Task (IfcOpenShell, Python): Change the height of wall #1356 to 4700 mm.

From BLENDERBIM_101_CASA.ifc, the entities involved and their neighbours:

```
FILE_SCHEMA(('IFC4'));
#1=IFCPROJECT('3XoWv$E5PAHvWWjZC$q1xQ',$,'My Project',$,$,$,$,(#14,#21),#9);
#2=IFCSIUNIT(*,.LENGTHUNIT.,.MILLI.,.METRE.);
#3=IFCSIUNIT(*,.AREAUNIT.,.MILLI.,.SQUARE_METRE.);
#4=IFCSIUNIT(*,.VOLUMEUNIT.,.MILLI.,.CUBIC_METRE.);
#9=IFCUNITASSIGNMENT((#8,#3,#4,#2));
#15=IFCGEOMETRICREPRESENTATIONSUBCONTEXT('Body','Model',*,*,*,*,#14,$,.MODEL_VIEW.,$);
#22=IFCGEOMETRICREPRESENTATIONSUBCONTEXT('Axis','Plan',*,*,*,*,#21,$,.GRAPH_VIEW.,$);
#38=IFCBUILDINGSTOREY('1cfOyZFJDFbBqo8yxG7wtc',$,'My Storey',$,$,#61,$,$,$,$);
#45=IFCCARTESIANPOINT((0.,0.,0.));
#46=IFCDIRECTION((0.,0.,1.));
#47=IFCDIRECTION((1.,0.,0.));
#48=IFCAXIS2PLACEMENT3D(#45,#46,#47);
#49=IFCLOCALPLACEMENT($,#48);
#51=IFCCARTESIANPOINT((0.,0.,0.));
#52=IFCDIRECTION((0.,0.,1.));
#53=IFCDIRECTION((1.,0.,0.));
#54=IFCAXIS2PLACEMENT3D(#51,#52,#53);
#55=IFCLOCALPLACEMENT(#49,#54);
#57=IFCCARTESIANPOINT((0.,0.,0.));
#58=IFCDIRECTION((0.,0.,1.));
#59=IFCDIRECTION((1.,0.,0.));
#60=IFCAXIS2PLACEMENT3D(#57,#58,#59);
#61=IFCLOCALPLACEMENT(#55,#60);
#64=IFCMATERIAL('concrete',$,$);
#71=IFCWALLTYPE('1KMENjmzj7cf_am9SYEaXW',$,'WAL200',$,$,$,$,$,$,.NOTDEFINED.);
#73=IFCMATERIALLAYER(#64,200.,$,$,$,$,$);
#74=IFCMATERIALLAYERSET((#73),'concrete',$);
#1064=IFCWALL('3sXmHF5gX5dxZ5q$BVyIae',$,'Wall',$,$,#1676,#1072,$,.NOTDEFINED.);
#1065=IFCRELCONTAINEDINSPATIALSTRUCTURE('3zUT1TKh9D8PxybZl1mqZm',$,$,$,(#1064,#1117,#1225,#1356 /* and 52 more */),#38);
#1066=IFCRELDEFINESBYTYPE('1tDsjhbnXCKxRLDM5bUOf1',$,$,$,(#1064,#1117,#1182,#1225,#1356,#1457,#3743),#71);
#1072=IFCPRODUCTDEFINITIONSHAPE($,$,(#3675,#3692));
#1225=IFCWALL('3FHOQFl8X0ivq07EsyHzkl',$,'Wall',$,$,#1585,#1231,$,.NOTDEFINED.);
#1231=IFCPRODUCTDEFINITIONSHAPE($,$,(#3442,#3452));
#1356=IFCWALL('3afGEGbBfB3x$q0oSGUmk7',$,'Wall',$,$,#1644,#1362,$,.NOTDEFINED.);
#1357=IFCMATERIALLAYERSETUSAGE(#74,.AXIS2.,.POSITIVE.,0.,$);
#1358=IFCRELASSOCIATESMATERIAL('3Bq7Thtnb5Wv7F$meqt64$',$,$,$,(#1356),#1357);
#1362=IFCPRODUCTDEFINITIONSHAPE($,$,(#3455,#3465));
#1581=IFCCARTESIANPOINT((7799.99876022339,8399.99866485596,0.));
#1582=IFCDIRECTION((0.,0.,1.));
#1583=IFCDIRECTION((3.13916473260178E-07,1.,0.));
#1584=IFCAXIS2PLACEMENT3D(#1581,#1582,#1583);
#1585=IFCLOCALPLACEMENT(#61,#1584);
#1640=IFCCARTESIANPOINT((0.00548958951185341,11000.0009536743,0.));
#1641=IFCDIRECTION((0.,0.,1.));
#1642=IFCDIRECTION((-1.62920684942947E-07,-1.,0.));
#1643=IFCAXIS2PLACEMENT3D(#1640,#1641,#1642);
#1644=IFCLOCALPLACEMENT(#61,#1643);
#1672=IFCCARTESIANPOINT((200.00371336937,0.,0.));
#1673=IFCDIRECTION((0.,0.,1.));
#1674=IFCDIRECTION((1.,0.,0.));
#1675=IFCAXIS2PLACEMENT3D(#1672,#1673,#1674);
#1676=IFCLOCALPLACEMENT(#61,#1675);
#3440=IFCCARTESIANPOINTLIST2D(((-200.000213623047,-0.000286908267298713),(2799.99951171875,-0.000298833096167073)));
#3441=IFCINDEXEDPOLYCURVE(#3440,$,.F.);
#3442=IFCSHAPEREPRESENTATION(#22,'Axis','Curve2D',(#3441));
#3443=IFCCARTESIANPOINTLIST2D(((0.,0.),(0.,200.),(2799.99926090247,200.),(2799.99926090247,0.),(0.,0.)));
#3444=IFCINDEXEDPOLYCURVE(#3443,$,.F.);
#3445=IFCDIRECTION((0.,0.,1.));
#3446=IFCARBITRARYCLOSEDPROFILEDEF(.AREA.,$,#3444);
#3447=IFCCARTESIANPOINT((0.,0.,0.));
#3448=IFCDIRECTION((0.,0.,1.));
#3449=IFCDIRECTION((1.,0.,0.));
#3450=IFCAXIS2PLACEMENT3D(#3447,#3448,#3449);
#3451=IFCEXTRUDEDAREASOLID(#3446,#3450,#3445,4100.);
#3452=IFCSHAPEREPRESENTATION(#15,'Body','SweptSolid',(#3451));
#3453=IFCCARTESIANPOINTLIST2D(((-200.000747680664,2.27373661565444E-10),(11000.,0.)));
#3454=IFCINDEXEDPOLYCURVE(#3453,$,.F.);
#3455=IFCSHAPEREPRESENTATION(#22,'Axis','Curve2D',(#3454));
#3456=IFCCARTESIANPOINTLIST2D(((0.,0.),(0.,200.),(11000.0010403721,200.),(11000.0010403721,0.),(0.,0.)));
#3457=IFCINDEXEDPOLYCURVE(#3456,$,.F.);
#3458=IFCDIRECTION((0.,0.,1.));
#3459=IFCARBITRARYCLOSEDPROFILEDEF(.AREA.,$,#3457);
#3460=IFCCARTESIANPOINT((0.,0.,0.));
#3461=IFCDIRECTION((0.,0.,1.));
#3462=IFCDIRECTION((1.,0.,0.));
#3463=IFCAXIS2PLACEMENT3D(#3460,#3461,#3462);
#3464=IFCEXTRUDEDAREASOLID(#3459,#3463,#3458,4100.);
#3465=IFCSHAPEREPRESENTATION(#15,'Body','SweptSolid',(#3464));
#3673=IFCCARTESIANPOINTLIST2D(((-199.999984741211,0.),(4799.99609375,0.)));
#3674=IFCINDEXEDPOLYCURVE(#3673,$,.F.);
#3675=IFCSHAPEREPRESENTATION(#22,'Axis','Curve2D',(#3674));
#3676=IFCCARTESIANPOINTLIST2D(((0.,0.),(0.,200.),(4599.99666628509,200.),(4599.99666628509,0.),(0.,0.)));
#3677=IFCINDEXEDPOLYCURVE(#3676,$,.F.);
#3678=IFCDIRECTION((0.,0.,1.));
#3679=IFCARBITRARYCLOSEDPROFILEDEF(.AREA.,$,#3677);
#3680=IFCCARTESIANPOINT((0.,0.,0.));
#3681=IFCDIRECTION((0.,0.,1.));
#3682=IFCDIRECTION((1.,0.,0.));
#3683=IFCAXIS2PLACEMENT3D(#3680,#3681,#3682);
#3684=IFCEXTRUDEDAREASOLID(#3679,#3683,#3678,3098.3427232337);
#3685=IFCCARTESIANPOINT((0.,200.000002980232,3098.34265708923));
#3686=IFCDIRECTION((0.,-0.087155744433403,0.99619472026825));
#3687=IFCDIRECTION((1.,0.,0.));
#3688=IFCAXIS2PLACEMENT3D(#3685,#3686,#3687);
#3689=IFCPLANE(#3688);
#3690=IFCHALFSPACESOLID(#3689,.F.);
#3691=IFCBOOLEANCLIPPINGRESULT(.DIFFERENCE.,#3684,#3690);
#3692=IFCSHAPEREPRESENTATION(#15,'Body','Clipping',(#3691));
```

```python
import ifcopenshell
import ifcopenshell.geom
import ifcopenshell.util.representation
import ifcopenshell.util.shape
import ifcopenshell.util.unit

model = ifcopenshell.open("BLENDERBIM_101_CASA.ifc")
unit_scale = ifcopenshell.util.unit.calculate_unit_scale(model)
settings = ifcopenshell.geom.settings()


def volume(element):
    """Net volume in cubic metres, openings subtracted."""
    shape = ifcopenshell.geom.create_shape(settings, element)
    return ifcopenshell.util.shape.get_volume(shape.geometry)


wall = model.by_id(1356)
before = volume(wall)

body = ifcopenshell.util.representation.get_representation(wall, "Model", "Body")
solid = body.Items[0]
old_height = solid.Depth
solid.Depth = 4.7 / unit_scale
after = volume(wall)

print(f"height {old_height:g} -> {solid.Depth:g}, volume {before:.3f} -> {after:.3f} m3")

model.write("BLENDERBIM_101_CASA_rev.ifc")
```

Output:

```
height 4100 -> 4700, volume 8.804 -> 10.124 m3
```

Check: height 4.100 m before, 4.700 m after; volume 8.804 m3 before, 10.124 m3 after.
